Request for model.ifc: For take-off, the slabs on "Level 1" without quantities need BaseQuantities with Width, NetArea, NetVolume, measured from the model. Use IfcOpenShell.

First a look at what the model holds.

```python
import ifcopenshell
import ifcopenshell.util.element
import ifcopenshell.util.unit

model = ifcopenshell.open("model.ifc")
print(model.schema)
for unit_type in ("LENGTHUNIT", "AREAUNIT", "VOLUMEUNIT"):
    print(unit_type, ifcopenshell.util.unit.calculate_unit_scale(model, unit_type))
storey = next(s for s in model.by_type("IfcBuildingStorey") if s.Name == "Level 1")
slabs = [e for e in ifcopenshell.util.element.get_decomposition(storey) if e.is_a("IfcSlab")]
for e in sorted(slabs, key=lambda e: e.id()):
    print(e.id(), e.is_a(), e.Name, list(ifcopenshell.util.element.get_psets(e, qtos_only=True)), sep=" | ")
```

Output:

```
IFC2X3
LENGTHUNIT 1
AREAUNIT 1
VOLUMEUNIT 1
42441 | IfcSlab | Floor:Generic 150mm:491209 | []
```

```python
import ifcopenshell
import ifcopenshell.api.pset
import ifcopenshell.geom
import ifcopenshell.util.element
import ifcopenshell.util.shape
import ifcopenshell.util.unit

model = ifcopenshell.open("model.ifc")
unit_scale = ifcopenshell.util.unit.calculate_unit_scale(model)
area_scale = ifcopenshell.util.unit.calculate_unit_scale(model, "AREAUNIT")
volume_scale = ifcopenshell.util.unit.calculate_unit_scale(model, "VOLUMEUNIT")
settings = ifcopenshell.geom.settings()

storey = next(s for s in model.by_type("IfcBuildingStorey") if s.Name == "Level 1")
slabs = [e for e in ifcopenshell.util.element.get_decomposition(storey) if e.is_a("IfcSlab")]

for e in sorted(slabs, key=lambda e: e.id()):
    if ifcopenshell.util.element.get_psets(e, qtos_only=True, should_inherit=False):
        continue
    # Geometry comes back in metres, in the element's own axes.
    shape = ifcopenshell.geom.create_shape(settings, e)
    values = {
        "Width": ifcopenshell.util.shape.get_z(shape.geometry) / unit_scale,
        "NetArea": ifcopenshell.util.shape.get_footprint_area(shape.geometry) / area_scale,
        "NetVolume": ifcopenshell.util.shape.get_volume(shape.geometry) / volume_scale,
    }
    qto = ifcopenshell.api.pset.add_qto(model, product=e, name="BaseQuantities")
    ifcopenshell.api.pset.edit_qto(model, qto=qto, properties=values)
    print(e.id(), {k: round(v, 3) for k, v in values.items()})

model.write("model-out.ifc")
```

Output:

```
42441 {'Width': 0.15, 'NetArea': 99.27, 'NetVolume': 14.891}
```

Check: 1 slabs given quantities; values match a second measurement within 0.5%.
